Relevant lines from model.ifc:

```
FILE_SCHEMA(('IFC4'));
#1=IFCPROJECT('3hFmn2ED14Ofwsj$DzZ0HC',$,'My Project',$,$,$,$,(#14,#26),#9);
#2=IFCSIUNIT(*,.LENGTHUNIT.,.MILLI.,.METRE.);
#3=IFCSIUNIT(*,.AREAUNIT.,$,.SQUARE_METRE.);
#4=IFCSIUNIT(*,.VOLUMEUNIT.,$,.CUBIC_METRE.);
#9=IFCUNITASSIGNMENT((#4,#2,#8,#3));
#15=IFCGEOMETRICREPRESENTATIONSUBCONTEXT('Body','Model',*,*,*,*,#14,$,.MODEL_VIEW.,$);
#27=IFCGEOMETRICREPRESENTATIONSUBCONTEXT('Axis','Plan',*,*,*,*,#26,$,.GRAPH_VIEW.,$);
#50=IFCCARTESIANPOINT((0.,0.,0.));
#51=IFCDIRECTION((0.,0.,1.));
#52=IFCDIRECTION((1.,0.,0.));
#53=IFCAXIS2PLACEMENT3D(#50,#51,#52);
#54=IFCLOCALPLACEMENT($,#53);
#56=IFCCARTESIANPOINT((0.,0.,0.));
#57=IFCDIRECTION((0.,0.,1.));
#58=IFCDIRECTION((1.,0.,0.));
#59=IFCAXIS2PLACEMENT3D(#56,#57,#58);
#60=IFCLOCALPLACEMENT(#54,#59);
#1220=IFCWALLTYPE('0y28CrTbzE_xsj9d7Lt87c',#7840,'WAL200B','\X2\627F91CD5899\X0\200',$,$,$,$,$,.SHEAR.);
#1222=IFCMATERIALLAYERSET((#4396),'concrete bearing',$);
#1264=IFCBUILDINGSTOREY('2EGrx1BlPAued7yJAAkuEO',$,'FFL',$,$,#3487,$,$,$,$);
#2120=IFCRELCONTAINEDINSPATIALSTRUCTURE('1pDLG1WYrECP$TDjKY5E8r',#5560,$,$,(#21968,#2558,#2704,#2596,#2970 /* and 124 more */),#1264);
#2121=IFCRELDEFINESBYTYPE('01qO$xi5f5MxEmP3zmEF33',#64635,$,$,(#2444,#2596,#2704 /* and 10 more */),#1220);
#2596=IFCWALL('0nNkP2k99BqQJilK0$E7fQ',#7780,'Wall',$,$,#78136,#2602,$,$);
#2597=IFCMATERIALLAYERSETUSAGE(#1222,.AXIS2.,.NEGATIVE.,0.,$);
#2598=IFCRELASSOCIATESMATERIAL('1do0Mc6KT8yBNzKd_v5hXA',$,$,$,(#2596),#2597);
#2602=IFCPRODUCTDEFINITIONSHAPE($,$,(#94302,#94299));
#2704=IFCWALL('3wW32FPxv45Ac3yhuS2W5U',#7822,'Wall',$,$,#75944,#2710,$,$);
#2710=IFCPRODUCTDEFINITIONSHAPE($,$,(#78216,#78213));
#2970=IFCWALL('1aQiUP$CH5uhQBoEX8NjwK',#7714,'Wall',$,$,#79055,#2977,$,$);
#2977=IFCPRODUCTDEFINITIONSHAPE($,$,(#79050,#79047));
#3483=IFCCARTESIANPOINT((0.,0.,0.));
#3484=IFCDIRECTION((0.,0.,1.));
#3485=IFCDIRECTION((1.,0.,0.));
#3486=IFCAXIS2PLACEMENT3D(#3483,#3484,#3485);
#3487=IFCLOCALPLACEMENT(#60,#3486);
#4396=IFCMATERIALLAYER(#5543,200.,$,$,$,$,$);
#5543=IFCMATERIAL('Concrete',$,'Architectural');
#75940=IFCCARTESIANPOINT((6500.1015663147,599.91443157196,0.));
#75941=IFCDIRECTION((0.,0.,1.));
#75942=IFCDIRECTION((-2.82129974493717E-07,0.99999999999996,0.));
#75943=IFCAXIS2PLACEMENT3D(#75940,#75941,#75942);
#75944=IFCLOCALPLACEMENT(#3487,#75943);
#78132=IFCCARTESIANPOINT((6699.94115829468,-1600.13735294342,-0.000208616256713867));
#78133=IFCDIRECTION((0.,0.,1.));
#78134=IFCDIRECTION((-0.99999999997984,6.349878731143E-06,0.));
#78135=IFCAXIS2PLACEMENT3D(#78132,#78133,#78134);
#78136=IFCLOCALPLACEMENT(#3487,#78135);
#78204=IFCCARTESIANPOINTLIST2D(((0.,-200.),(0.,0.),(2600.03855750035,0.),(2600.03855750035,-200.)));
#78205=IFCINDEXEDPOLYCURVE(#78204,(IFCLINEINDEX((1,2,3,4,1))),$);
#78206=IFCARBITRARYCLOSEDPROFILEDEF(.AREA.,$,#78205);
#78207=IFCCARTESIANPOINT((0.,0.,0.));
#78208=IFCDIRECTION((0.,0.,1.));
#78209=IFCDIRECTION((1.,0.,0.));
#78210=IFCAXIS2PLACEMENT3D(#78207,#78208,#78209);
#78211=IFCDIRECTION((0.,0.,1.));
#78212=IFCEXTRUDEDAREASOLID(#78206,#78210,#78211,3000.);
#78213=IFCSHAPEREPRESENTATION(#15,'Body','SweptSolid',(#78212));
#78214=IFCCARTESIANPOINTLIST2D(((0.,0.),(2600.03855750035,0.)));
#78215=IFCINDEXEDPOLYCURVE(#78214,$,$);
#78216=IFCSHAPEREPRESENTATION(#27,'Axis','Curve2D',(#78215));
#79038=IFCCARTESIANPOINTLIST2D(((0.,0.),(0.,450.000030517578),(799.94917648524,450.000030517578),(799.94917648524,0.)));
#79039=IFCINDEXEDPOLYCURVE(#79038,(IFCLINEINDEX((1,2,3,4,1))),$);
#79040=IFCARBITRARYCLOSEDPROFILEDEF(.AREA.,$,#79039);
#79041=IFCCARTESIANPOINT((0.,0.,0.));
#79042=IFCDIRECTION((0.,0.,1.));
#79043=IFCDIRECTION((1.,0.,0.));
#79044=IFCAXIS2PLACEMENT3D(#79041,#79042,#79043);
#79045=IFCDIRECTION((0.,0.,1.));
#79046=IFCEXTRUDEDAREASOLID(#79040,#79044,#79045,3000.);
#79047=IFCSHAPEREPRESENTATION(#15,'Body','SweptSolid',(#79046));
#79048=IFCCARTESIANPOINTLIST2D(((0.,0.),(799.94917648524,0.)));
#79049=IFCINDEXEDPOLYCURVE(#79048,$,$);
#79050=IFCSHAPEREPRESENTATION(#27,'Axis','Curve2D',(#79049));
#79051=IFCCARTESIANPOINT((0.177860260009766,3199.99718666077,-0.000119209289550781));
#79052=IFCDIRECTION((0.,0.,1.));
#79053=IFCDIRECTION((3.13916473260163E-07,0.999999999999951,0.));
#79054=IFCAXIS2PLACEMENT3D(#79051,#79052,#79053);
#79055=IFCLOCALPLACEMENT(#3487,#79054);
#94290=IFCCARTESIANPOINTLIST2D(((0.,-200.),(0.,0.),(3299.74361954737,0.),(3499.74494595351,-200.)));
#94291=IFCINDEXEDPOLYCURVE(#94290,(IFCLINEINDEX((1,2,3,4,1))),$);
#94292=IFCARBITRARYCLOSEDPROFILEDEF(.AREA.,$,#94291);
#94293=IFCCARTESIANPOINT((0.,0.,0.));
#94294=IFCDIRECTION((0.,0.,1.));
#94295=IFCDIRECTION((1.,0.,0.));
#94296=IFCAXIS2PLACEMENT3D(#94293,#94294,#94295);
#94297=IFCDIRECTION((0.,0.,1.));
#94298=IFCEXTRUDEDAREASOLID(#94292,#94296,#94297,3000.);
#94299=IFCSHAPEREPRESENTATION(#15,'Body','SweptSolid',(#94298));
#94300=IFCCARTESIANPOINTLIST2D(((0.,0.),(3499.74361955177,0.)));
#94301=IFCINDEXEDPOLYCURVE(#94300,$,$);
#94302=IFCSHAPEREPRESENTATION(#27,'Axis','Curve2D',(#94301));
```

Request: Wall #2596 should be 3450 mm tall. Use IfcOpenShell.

```python
import ifcopenshell
import ifcopenshell.geom
import ifcopenshell.util.representation
import ifcopenshell.util.shape
import ifcopenshell.util.unit

model = ifcopenshell.open("model.ifc")
unit_scale = ifcopenshell.util.unit.calculate_unit_scale(model)
settings = ifcopenshell.geom.settings()


def volume(element):
    """Net volume in cubic metres, openings subtracted."""
    shape = ifcopenshell.geom.create_shape(settings, element)
    return ifcopenshell.util.shape.get_volume(shape.geometry)


wall = model.by_guid("0nNkP2k99BqQJilK0$E7fQ")
before = volume(wall)

body = ifcopenshell.util.representation.get_representation(wall, "Model", "Body")
solid = body.Items[0]
old_height = solid.Depth
solid.Depth = 3.45 / unit_scale
after = volume(wall)

print(f"height {old_height:g} -> {solid.Depth:g}, volume {before:.3f} -> {after:.3f} m3")

model.write("model_v2.ifc")
```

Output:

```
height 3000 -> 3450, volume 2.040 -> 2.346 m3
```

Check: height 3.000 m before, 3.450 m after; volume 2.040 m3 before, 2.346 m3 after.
